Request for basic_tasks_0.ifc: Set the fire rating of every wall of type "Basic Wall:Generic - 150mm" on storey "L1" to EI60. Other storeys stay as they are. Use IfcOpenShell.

First a look at what the model holds.

```python
import ifcopenshell
import ifcopenshell.util.element

model = ifcopenshell.open("basic_tasks_0.ifc")
print(model.schema)
storey = next(s for s in model.by_type("IfcBuildingStorey") if s.Name == "L1")
walls = [e for e in ifcopenshell.util.element.get_decomposition(storey) if e.is_a("IfcWall")]
seen = {}
for e in walls:
    element_type = ifcopenshell.util.element.get_type(e)
    key = (element_type.Name if element_type != e and element_type else None, ifcopenshell.util.element.get_pset(e, "Pset_WallCommon", "FireRating"))
    seen[key] = seen.get(key, 0) + 1
for (name, value), count in sorted(seen.items(), key=str):
    print(count, "x", name, "|", value)
```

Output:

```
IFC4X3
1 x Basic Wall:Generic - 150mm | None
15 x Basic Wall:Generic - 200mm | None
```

```python
import ifcopenshell
import ifcopenshell.api.pset
import ifcopenshell.util.element

model = ifcopenshell.open("basic_tasks_0.ifc")

storey = next(s for s in model.by_type("IfcBuildingStorey") if s.Name == "L1")
walls = [e for e in ifcopenshell.util.element.get_decomposition(storey) if e.is_a("IfcWall")]

count = 0
for e in walls:
    element_type = ifcopenshell.util.element.get_type(e)
    if element_type in (None, e) or element_type.Name != "Basic Wall:Generic - 150mm":
        continue
    # add_pset returns the element's existing set when there is one.
    pset = ifcopenshell.api.pset.add_pset(model, product=e, name="Pset_WallCommon")
    ifcopenshell.api.pset.edit_pset(model, pset=pset, properties={"FireRating": "EI60"})
    count += 1

print(count, "walls updated")

model.write("basic_tasks_0_updated.ifc")
```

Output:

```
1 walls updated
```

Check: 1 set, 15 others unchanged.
